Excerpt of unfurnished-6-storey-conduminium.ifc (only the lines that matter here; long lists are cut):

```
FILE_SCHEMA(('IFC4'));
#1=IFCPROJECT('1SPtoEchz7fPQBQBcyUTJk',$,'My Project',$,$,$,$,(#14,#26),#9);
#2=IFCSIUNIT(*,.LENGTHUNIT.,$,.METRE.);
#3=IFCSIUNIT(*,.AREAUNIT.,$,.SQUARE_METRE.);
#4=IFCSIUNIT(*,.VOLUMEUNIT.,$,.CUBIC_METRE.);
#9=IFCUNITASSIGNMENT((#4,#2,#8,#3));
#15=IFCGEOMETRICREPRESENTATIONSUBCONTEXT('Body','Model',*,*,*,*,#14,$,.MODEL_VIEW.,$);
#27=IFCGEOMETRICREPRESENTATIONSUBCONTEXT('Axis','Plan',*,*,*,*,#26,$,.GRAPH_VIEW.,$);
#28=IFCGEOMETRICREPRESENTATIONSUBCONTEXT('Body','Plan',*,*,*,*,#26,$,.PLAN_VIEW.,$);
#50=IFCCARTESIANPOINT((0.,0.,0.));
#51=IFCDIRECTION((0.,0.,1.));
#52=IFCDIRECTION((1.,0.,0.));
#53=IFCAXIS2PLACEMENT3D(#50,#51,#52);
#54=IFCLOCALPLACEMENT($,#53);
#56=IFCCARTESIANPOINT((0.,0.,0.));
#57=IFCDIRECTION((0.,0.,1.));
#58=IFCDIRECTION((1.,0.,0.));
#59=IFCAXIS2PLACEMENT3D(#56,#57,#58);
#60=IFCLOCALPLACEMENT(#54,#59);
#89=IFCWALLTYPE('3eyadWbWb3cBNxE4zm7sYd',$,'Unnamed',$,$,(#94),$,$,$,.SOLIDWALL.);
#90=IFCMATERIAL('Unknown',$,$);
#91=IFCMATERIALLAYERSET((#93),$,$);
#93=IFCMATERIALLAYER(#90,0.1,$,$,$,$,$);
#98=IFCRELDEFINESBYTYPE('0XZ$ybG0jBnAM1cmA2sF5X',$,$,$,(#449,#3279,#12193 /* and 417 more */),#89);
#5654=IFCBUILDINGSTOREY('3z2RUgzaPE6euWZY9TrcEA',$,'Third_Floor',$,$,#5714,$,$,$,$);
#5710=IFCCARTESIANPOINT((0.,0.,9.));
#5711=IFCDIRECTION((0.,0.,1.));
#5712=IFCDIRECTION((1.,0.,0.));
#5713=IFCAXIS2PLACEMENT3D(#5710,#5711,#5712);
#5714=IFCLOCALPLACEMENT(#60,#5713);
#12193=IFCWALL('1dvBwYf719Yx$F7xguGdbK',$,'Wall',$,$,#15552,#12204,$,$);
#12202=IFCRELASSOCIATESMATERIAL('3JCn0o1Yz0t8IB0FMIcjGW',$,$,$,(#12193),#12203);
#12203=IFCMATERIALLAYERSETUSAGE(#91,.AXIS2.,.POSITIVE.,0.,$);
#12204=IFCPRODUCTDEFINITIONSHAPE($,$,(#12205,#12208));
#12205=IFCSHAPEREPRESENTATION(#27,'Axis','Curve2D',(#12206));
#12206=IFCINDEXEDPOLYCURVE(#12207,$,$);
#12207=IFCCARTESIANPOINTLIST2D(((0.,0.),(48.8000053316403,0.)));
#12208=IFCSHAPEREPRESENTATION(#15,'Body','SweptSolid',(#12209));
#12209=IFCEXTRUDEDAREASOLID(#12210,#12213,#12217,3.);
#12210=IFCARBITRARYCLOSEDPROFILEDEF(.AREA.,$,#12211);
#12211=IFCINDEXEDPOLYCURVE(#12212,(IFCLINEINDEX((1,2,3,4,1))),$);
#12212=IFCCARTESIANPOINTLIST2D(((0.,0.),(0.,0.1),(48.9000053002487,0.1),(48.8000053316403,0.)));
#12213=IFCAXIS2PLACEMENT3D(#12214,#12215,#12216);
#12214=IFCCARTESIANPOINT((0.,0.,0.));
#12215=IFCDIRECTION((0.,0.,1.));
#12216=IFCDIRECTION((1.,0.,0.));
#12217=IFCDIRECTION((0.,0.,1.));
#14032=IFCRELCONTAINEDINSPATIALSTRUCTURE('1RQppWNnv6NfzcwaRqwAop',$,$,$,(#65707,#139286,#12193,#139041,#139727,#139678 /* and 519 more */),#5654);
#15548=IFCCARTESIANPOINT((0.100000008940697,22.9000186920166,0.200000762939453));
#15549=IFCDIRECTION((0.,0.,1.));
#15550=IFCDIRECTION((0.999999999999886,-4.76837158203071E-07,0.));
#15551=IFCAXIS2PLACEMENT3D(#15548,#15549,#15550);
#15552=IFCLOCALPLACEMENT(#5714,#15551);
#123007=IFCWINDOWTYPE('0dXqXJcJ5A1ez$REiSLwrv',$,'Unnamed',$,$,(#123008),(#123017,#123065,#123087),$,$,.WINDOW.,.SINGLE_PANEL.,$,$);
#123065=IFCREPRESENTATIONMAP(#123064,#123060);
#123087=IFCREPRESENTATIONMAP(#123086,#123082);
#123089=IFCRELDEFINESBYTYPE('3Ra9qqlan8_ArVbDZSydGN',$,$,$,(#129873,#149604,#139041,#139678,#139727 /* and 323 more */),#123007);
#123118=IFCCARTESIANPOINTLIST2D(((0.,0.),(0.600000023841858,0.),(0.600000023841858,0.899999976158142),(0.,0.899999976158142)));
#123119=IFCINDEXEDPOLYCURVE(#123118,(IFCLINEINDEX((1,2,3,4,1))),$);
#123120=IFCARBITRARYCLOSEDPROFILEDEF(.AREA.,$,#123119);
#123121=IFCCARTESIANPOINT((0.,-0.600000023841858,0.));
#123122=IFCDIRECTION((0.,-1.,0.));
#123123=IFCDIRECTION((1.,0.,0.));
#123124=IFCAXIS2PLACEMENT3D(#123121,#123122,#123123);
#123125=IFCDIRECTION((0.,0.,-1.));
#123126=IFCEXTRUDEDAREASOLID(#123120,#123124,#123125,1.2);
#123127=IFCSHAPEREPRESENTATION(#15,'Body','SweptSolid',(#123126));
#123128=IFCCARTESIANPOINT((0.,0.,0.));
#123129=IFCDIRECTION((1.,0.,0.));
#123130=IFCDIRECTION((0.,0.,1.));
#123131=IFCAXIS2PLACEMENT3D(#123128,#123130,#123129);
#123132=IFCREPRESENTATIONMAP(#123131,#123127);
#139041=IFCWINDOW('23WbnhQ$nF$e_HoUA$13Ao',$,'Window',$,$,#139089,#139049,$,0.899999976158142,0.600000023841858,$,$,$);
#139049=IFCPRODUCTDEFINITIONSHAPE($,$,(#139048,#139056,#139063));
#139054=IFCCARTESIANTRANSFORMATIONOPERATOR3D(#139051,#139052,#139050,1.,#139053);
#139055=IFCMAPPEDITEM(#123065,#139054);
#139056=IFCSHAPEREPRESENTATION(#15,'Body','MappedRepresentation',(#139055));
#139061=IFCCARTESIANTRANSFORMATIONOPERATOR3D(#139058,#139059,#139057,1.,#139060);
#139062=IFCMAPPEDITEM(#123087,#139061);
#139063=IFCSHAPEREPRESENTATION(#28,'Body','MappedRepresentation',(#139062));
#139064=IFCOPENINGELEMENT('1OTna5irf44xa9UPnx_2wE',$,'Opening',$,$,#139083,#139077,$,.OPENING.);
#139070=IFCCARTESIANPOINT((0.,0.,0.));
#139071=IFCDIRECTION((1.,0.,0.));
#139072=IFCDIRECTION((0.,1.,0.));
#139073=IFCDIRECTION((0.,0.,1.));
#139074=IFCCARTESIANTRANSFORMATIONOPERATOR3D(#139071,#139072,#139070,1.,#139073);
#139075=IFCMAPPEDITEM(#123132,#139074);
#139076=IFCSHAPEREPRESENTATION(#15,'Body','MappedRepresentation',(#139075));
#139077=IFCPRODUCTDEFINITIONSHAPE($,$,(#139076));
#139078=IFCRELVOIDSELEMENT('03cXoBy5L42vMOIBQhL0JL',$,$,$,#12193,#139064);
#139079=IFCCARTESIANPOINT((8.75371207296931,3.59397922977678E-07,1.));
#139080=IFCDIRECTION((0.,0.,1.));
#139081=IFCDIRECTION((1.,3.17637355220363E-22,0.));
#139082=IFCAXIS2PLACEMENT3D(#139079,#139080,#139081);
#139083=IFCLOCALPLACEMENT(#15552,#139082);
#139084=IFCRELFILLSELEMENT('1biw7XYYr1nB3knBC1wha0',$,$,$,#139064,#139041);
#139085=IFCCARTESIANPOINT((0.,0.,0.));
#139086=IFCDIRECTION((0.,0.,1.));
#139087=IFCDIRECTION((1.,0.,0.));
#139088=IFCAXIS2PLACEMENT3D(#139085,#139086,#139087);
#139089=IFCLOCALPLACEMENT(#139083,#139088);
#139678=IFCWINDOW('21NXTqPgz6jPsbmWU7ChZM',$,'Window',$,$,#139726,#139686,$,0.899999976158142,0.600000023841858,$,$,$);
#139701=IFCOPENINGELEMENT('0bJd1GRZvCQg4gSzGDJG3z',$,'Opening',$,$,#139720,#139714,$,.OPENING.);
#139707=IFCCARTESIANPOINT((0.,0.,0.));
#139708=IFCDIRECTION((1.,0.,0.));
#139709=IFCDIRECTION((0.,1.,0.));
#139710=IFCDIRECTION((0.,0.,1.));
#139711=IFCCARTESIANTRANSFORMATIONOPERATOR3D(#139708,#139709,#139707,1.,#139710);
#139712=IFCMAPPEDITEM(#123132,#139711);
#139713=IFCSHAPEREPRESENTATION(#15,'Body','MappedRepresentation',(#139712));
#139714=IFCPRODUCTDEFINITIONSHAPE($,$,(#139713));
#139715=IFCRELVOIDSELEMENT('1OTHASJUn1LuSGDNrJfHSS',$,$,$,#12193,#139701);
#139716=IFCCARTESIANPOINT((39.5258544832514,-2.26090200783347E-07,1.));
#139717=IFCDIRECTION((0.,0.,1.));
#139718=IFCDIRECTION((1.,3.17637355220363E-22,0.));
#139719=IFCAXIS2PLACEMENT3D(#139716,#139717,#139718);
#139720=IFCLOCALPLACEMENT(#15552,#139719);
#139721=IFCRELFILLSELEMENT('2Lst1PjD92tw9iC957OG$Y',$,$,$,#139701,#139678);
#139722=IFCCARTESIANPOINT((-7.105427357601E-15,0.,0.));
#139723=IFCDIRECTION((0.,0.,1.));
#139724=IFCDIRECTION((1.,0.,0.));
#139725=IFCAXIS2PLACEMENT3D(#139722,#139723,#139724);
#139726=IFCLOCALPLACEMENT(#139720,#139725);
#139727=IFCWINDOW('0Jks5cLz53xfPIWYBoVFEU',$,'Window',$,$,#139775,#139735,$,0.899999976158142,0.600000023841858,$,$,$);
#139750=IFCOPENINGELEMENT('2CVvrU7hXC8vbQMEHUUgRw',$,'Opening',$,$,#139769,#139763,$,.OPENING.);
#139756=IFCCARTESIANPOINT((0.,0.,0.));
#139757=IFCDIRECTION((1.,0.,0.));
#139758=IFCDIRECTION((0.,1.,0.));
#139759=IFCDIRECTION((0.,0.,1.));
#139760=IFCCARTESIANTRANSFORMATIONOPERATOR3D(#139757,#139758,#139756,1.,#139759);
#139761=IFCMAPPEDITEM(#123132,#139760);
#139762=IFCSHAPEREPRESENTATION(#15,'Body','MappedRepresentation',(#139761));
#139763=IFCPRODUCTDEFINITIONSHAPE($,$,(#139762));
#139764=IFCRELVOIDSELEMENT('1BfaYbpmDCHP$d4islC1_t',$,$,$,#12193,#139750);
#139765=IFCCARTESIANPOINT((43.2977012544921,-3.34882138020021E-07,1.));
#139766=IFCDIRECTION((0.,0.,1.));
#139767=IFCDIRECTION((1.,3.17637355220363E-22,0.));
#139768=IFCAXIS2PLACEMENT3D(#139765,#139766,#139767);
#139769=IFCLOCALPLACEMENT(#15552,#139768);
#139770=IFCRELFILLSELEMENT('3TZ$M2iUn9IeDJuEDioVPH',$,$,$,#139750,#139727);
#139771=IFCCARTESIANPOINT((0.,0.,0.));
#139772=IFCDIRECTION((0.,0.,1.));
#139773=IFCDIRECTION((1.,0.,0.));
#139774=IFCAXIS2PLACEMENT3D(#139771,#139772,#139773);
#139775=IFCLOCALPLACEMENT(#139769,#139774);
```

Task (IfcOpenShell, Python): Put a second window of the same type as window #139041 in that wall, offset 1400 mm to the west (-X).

```python
import ifcopenshell
import ifcopenshell.api.feature
import ifcopenshell.api.geometry
import ifcopenshell.api.root
import ifcopenshell.geom
import ifcopenshell.util.element
import ifcopenshell.util.placement
import ifcopenshell.util.shape
import ifcopenshell.util.unit

model = ifcopenshell.open("unfurnished-6-storey-conduminium.ifc")
unit_scale = ifcopenshell.util.unit.calculate_unit_scale(model)
settings = ifcopenshell.geom.settings()


def volume(element):
    """Net volume in cubic metres, openings subtracted."""
    shape = ifcopenshell.geom.create_shape(settings, element)
    return ifcopenshell.util.shape.get_volume(shape.geometry)


window = model.by_guid("23WbnhQ$nF$e_HoUA$13Ao")
opening = window.FillsVoids[0].RelatingOpeningElement
wall = opening.VoidsElements[0].RelatingBuildingElement
before = volume(wall)
shift = ifcopenshell.util.placement.get_local_placement(wall.ObjectPlacement)[:3, 0] * -1.4 / unit_scale

# copy_class copies the void relationship, type, container and properties, but no geometry.
new_opening = ifcopenshell.api.root.copy_class(model, product=opening)
new_opening.Representation = ifcopenshell.util.element.copy_deep(
    model, opening.Representation, exclude=["IfcGeometricRepresentationContext", "IfcRepresentationMap"]
)
new_window = ifcopenshell.api.root.copy_class(model, product=window)
new_window.Representation = ifcopenshell.util.element.copy_deep(
    model, window.Representation, exclude=["IfcGeometricRepresentationContext", "IfcRepresentationMap"]
)
ifcopenshell.api.feature.add_filling(model, opening=new_opening, element=new_window)

for old, new in ((opening, new_opening), (window, new_window)):
    matrix = ifcopenshell.util.placement.get_local_placement(old.ObjectPlacement)
    matrix[:3, 3] += shift
    ifcopenshell.api.geometry.edit_object_placement(model, product=new, matrix=matrix, is_si=False)

after = volume(wall)

print(f"wall volume {before:.3f} -> {after:.3f} m3")

model.write("unfurnished-6-storey-conduminium_updated.ifc")
```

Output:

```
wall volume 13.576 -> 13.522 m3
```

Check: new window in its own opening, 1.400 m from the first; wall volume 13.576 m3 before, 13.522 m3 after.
